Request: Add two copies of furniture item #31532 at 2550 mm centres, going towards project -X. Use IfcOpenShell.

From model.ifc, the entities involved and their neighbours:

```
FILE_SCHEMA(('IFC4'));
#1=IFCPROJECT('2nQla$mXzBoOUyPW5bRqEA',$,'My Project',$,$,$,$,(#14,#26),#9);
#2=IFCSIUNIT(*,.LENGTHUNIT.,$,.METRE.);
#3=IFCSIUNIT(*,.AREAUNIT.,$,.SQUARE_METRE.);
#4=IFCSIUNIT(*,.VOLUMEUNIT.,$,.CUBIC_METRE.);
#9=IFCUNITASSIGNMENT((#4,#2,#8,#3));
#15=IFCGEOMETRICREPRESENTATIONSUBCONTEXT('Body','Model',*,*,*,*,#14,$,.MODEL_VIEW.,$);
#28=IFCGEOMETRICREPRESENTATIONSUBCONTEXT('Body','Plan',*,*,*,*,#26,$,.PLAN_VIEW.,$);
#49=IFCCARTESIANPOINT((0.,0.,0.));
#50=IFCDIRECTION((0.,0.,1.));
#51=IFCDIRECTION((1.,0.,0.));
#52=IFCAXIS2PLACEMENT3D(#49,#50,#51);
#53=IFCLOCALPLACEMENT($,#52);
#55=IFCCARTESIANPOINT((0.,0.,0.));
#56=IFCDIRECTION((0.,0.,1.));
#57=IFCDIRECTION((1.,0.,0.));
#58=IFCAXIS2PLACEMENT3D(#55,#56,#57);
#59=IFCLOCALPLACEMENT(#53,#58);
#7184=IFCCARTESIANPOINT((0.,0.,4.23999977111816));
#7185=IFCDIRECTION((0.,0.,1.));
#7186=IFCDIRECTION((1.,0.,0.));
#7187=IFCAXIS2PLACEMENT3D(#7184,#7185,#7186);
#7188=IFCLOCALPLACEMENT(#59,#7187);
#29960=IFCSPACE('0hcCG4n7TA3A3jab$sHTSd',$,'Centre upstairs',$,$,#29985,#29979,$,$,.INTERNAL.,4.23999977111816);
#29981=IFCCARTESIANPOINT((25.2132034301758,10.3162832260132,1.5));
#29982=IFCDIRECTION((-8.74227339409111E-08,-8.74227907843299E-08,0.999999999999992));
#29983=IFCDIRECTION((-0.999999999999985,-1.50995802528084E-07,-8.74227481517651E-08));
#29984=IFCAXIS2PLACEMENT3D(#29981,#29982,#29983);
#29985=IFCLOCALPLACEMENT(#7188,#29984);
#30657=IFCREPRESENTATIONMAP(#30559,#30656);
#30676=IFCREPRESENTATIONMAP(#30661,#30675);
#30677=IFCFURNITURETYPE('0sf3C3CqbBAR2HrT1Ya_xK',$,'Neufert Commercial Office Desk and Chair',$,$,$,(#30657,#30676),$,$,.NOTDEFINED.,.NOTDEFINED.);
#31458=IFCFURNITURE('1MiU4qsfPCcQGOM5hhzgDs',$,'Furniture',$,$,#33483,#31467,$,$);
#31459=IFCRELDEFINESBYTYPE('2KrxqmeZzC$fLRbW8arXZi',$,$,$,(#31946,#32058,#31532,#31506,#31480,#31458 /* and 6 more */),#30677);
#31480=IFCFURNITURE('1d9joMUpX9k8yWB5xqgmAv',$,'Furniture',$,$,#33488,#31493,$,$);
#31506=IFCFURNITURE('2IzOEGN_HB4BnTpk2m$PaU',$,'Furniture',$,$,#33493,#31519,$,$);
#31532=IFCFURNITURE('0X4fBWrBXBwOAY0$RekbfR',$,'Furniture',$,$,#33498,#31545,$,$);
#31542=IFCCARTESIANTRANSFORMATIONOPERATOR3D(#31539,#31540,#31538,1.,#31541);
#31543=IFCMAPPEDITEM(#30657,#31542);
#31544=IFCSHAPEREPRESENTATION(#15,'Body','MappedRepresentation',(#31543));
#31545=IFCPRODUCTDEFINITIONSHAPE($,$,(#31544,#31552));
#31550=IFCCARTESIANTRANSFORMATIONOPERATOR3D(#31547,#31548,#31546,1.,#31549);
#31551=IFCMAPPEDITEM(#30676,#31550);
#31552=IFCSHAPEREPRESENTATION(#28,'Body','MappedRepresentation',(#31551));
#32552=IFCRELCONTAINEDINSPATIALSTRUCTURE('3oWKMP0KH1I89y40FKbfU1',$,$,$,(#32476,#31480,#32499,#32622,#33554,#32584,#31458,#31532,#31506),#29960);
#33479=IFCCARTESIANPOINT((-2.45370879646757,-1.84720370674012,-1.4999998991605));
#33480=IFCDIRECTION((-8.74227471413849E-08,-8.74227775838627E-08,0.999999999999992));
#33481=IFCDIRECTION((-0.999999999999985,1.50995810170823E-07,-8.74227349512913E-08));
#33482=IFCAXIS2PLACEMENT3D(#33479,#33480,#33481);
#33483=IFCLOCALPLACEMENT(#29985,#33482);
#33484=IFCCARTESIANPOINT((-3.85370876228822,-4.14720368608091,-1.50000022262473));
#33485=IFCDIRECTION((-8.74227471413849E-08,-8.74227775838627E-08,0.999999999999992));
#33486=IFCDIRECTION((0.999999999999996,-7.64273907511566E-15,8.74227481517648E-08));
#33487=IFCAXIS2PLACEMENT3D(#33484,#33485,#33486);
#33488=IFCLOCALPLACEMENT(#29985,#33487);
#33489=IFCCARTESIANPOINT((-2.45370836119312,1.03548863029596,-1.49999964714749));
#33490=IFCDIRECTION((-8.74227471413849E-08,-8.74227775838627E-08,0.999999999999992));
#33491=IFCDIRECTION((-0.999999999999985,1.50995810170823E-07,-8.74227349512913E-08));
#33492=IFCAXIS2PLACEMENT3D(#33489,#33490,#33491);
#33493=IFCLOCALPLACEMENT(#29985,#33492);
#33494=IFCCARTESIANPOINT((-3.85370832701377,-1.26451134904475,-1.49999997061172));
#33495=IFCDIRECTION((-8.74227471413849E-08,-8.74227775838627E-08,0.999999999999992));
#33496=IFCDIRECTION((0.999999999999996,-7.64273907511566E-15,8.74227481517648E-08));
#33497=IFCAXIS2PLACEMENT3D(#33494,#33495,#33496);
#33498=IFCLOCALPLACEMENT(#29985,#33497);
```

```python
import numpy as np
import ifcopenshell
import ifcopenshell.api.geometry
import ifcopenshell.api.root
import ifcopenshell.util.element
import ifcopenshell.util.placement

model = ifcopenshell.open("model.ifc")

source = model.by_id(31532)
base = ifcopenshell.util.placement.get_local_placement(source.ObjectPlacement)
step = np.array([-1.0, 0.0, 0.0]) * 2.55

for i in range(1, 3):
    copy = ifcopenshell.api.root.copy_class(model, product=source)
    copy.Representation = ifcopenshell.util.element.copy_deep(
        model, source.Representation, exclude=["IfcGeometricRepresentationContext", "IfcRepresentationMap"]
    )
    matrix = base.copy()
    matrix[:3, 3] += i * step
    print("added at", matrix[:3, 3].round(3) + 0.0)
    ifcopenshell.api.geometry.edit_object_placement(model, product=copy, matrix=matrix, is_si=False)

model.write("model_rev.ifc")
```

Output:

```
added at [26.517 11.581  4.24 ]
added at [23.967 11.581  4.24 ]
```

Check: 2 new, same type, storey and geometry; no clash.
